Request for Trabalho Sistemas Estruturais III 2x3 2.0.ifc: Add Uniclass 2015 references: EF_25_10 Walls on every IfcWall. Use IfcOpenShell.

First a look at what the model holds.

```python
import ifcopenshell

model = ifcopenshell.open("Trabalho Sistemas Estruturais III 2x3 2.0.ifc")
print(model.schema)
print("classifications:", [c.Name for c in model.by_type("IfcClassification")])
for ifc_class in ("IfcDoor", "IfcRoof", "IfcStair", "IfcWall", "IfcWindow"):
    print(ifc_class, len(model.by_type(ifc_class)))
```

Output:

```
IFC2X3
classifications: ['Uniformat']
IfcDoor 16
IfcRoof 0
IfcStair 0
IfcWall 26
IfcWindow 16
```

```python
import ifcopenshell
import ifcopenshell.api.classification

model = ifcopenshell.open("Trabalho Sistemas Estruturais III 2x3 2.0.ifc")

# IFC2X3 requires Source and Edition and has no link from the project to the system.
system = model.create_entity("IfcClassification", Source="NBS", Edition="2015", Name="Uniclass 2015")

codes = {
    "IfcWall": ("EF_25_10", "Walls"),
}
for ifc_class, (code, name) in codes.items():
    products = model.by_type(ifc_class)
    ifcopenshell.api.classification.add_reference(
        model, products=products, classification=system, identification=code, name=name
    )
    print(code, len(products))

model.write("Trabalho Sistemas Estruturais III 2x3 2.0_v2.ifc")
```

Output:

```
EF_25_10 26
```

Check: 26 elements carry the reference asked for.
